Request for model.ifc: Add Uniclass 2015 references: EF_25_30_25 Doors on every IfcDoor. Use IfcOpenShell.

First a look at what the model holds.

```python
import ifcopenshell

model = ifcopenshell.open("model.ifc")
print(model.schema)
print("classifications:", [c.Name for c in model.by_type("IfcClassification")])
for ifc_class in ("IfcDoor", "IfcRoof", "IfcStair", "IfcWall", "IfcWindow"):
    print(ifc_class, len(model.by_type(ifc_class)))
```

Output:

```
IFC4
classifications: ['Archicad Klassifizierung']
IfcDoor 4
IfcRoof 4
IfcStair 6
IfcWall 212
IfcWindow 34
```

```python
import ifcopenshell
import ifcopenshell.api.classification

model = ifcopenshell.open("model.ifc")

system = ifcopenshell.api.classification.add_classification(model, classification="Uniclass 2015")

codes = {
    "IfcDoor": ("EF_25_30_25", "Doors"),
}
for ifc_class, (code, name) in codes.items():
    products = model.by_type(ifc_class)
    ifcopenshell.api.classification.add_reference(
        model, products=products, classification=system, identification=code, name=name
    )
    print(code, len(products))

model.write("model_edited.ifc")
```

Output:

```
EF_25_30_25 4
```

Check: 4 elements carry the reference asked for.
